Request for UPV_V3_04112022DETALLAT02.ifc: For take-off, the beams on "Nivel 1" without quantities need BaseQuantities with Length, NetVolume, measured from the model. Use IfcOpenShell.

First a look at what the model holds.

```python
import ifcopenshell
import ifcopenshell.util.element
import ifcopenshell.util.unit

model = ifcopenshell.open("UPV_V3_04112022DETALLAT02.ifc")
print(model.schema)
for unit_type in ("LENGTHUNIT", "AREAUNIT", "VOLUMEUNIT"):
    print(unit_type, ifcopenshell.util.unit.calculate_unit_scale(model, unit_type))
storey = next(s for s in model.by_type("IfcBuildingStorey") if s.Name == "Nivel 1")
beams = [e for e in ifcopenshell.util.element.get_decomposition(storey) if e.is_a("IfcBeam")]
for e in sorted(beams, key=lambda e: e.id()):
    print(e.id(), e.is_a(), e.Name, list(ifcopenshell.util.element.get_psets(e, qtos_only=True)), sep=" | ")
```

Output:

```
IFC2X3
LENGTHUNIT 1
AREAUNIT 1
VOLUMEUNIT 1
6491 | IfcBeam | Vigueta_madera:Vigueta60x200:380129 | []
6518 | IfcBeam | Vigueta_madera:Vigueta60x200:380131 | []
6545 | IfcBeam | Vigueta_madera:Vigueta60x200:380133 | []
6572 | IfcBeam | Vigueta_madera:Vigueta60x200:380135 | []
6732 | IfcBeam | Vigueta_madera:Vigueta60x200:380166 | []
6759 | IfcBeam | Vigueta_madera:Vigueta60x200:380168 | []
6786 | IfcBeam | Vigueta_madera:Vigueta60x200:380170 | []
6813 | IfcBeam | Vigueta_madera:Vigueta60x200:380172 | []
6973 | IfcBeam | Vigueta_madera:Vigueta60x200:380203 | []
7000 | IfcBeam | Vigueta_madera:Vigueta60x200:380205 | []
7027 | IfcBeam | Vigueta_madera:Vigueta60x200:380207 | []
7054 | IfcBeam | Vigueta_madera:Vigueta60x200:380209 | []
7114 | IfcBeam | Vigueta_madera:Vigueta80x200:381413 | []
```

```python
import ifcopenshell
import ifcopenshell.api.pset
import ifcopenshell.geom
import ifcopenshell.util.element
import ifcopenshell.util.shape
import ifcopenshell.util.unit

model = ifcopenshell.open("UPV_V3_04112022DETALLAT02.ifc")
unit_scale = ifcopenshell.util.unit.calculate_unit_scale(model)
volume_scale = ifcopenshell.util.unit.calculate_unit_scale(model, "VOLUMEUNIT")
settings = ifcopenshell.geom.settings()

storey = next(s for s in model.by_type("IfcBuildingStorey") if s.Name == "Nivel 1")
beams = [e for e in ifcopenshell.util.element.get_decomposition(storey) if e.is_a("IfcBeam")]

for e in sorted(beams, key=lambda e: e.id()):
    if ifcopenshell.util.element.get_psets(e, qtos_only=True, should_inherit=False):
        continue
    # Geometry comes back in metres, in the element's own axes.
    shape = ifcopenshell.geom.create_shape(settings, e)
    values = {
        "Length": ifcopenshell.util.shape.get_max_xyz(shape.geometry) / unit_scale,
        "NetVolume": ifcopenshell.util.shape.get_volume(shape.geometry) / volume_scale,
    }
    qto = ifcopenshell.api.pset.add_qto(model, product=e, name="BaseQuantities")
    ifcopenshell.api.pset.edit_qto(model, qto=qto, properties=values)
    print(e.id(), {k: round(v, 3) for k, v in values.items()})

model.write("UPV_V3_04112022DETALLAT02_rev.ifc")
```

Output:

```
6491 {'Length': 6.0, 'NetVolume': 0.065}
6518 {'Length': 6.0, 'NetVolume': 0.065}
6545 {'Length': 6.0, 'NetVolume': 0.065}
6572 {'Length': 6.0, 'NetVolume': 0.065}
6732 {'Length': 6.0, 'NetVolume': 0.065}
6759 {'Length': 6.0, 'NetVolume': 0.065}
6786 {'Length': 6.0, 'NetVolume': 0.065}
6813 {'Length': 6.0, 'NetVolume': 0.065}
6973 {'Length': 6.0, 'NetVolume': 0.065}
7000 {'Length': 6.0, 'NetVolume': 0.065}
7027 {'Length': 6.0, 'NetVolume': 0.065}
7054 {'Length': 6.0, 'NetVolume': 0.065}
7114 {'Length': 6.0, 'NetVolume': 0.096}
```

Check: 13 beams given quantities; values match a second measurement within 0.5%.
